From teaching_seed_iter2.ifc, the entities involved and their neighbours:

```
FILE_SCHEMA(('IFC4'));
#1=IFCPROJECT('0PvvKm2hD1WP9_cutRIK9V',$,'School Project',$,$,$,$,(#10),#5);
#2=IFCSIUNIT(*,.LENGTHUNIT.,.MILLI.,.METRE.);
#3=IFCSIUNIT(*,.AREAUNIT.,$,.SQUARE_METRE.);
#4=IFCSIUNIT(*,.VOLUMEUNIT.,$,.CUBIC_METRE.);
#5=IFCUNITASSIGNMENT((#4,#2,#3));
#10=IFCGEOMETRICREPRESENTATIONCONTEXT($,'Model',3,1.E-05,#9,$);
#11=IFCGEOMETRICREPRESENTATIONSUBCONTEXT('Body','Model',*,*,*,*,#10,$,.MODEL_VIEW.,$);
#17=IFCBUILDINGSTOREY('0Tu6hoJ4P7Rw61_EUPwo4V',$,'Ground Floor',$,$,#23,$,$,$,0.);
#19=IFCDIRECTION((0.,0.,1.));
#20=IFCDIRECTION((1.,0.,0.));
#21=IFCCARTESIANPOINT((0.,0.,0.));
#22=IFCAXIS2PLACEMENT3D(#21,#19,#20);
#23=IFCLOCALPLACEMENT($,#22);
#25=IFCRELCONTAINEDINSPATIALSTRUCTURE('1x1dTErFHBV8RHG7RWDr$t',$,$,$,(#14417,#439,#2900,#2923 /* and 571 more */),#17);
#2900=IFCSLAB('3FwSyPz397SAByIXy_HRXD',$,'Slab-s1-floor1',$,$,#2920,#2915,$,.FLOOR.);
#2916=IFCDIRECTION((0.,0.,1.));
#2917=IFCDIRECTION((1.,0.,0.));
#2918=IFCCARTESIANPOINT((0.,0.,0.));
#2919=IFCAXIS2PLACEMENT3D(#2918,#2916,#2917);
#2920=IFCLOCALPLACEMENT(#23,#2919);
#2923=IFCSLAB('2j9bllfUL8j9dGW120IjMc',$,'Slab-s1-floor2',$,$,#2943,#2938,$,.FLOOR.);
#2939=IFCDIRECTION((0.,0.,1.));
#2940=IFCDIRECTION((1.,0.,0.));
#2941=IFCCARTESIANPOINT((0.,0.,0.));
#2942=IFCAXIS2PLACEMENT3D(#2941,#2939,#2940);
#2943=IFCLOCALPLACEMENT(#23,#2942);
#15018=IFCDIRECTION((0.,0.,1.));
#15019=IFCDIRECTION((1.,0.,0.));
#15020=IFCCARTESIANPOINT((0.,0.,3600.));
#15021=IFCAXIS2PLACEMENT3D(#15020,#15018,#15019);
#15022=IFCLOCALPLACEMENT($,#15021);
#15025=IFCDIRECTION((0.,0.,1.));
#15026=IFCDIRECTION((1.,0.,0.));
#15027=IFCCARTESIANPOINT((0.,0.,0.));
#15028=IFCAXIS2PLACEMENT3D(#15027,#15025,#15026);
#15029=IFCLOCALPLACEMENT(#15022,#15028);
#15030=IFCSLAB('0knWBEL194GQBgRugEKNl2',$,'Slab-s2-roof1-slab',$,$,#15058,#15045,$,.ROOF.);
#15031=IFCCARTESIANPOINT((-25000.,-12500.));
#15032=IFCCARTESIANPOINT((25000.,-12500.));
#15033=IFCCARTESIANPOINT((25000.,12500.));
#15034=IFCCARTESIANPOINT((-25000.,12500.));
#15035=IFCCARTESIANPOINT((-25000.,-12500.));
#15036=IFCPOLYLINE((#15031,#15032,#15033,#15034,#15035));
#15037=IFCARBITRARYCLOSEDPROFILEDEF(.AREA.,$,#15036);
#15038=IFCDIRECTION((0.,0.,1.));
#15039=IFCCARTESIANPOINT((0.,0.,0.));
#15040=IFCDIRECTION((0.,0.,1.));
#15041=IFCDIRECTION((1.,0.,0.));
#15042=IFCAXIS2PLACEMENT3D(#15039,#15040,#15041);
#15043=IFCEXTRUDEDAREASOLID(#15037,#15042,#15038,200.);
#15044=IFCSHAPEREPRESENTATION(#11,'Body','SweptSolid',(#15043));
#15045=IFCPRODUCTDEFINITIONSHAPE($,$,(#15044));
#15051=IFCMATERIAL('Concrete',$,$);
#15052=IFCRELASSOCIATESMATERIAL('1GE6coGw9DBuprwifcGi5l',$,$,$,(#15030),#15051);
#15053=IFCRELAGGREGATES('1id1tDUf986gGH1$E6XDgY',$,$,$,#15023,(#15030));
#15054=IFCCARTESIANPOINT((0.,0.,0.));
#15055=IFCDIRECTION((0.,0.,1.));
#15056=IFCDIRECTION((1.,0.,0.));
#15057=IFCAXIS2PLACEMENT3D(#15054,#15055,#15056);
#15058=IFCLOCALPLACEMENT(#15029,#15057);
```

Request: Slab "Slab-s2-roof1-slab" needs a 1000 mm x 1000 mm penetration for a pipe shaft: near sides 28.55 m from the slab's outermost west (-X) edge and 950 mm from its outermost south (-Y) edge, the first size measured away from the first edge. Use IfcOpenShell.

```python
import numpy as np
import ifcopenshell
import ifcopenshell.api.feature
import ifcopenshell.api.geometry
import ifcopenshell.api.root
import ifcopenshell.geom
import ifcopenshell.util.placement
import ifcopenshell.util.representation
import ifcopenshell.util.shape
import ifcopenshell.util.unit

model = ifcopenshell.open("teaching_seed_iter2.ifc")
unit_scale = ifcopenshell.util.unit.calculate_unit_scale(model)
settings = ifcopenshell.geom.settings()


def volume(element):
    """Net volume in cubic metres, openings subtracted."""
    shape = ifcopenshell.geom.create_shape(settings, element)
    return ifcopenshell.util.shape.get_volume(shape.geometry)


slab = model.by_id(15030)
before = volume(slab)

# Extent in the slab's own axes, in metres. The edges named are its -X and -Y sides.
slab_shape = ifcopenshell.geom.create_shape(settings, slab)
vertices = ifcopenshell.util.shape.get_vertices(slab_shape.geometry)
x_min, y_min, bottom = vertices.min(axis=0)
top = vertices[:, 2].max()

opening = ifcopenshell.api.root.create_entity(model, ifc_class="IfcOpeningElement", name="Pipe shaft opening", predefined_type="OPENING")
context = ifcopenshell.util.representation.get_context(model, "Model", "Body", "MODEL_VIEW")
width, depth = 1, 1
outline = [(0.0, 0.0), (width, 0.0), (width, depth), (0.0, depth), (0.0, 0.0)]
# Overshoot both faces by 50 mm so the cut is clean.
shape = ifcopenshell.api.geometry.add_slab_representation(
    model, context=context, depth=top - bottom + 0.1, polyline=outline
)
ifcopenshell.api.geometry.assign_representation(model, product=opening, representation=shape)

matrix = ifcopenshell.util.placement.get_local_placement(slab.ObjectPlacement)
matrix[:, 3] = matrix @ np.append(np.array([x_min + 28.55, y_min + 0.95, bottom - 0.05]) / unit_scale, 1.0)
ifcopenshell.api.geometry.edit_object_placement(model, product=opening, matrix=matrix, is_si=False)
ifcopenshell.api.feature.add_feature(model, feature=opening, element=slab)

after = volume(slab)

print(f"slab volume {before:.3f} -> {after:.3f} m3")

model.write("teaching_seed_iter2-out.ifc")
```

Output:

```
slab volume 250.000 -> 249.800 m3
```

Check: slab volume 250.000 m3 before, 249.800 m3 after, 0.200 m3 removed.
